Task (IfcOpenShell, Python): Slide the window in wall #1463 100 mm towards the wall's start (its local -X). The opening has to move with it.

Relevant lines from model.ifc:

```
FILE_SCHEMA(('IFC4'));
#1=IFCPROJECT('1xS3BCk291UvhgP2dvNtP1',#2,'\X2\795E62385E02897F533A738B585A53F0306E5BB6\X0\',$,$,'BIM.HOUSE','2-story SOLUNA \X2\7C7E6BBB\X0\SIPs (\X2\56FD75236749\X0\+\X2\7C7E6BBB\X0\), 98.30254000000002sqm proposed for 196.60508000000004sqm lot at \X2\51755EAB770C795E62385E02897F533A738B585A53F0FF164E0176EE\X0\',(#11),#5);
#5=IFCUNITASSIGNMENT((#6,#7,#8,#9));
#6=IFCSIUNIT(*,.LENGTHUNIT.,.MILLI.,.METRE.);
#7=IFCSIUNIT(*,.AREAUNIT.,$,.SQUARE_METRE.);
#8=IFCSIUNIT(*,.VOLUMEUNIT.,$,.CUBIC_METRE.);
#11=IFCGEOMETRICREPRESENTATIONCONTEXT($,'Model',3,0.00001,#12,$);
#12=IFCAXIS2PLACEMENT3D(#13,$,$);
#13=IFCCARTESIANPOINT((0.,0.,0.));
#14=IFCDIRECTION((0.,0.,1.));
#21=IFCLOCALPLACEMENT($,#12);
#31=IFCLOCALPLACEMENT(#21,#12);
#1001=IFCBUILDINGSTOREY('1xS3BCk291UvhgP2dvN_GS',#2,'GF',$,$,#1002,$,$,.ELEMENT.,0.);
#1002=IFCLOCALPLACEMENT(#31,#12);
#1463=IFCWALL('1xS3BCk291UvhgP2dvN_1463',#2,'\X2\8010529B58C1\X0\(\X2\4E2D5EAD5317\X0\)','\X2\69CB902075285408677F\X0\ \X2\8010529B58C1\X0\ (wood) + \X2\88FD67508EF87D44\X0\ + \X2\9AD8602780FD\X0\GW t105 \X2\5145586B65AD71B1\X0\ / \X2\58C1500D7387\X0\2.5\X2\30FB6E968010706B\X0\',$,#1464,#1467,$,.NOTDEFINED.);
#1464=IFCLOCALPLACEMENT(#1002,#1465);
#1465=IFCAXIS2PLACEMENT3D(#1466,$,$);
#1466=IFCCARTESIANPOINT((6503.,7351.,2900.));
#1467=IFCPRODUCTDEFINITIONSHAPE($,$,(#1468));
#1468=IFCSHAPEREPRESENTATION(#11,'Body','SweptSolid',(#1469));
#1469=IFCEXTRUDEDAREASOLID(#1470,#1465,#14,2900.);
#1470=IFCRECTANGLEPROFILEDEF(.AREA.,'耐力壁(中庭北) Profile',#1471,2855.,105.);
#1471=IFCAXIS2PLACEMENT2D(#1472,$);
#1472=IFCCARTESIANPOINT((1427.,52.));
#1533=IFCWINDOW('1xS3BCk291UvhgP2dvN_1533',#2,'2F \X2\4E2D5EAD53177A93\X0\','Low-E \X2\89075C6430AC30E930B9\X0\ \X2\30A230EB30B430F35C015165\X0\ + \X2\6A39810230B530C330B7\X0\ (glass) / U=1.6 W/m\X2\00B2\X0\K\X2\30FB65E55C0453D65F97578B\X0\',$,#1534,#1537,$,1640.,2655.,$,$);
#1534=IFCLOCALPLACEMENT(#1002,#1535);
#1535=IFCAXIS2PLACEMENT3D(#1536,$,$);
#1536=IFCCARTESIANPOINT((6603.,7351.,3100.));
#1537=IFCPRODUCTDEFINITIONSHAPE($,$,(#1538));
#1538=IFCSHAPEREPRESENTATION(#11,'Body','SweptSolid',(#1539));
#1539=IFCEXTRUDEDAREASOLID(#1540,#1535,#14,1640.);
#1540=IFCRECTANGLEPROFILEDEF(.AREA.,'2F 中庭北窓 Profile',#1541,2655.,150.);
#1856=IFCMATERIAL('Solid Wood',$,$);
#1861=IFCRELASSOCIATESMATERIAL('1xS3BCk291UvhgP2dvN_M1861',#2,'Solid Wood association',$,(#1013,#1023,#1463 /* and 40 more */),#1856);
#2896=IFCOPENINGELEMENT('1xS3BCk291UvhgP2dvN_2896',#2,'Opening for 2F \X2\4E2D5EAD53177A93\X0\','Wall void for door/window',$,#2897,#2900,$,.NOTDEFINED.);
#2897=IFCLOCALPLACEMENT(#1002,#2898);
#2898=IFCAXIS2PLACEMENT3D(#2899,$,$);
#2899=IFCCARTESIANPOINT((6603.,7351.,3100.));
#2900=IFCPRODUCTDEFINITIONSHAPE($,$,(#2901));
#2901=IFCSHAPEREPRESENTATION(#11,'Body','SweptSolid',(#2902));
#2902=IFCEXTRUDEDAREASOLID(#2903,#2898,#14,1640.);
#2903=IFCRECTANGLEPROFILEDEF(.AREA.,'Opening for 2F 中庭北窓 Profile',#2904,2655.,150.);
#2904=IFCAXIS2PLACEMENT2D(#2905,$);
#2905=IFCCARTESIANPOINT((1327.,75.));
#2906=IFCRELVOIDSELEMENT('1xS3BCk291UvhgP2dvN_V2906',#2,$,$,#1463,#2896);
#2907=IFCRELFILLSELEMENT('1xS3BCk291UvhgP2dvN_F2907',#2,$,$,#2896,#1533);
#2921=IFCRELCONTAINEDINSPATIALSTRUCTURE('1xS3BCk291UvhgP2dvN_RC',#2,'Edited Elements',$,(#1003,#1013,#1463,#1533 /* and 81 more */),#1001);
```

```python
import ifcopenshell
import ifcopenshell.api.geometry
import ifcopenshell.util.placement

model = ifcopenshell.open("model.ifc")

window = model.by_id(1533)
opening = window.FillsVoids[0].RelatingOpeningElement
wall = opening.VoidsElements[0].RelatingBuildingElement

wall_matrix = ifcopenshell.util.placement.get_local_placement(wall.ObjectPlacement)
shift = wall_matrix[:3, 0] * -100.0
before = ifcopenshell.util.placement.get_local_placement(window.ObjectPlacement)[:3, 3].copy()

# The window is not placed relative to its opening, so move both.
for product in (opening, window):
    matrix = ifcopenshell.util.placement.get_local_placement(product.ObjectPlacement)
    matrix[:3, 3] += shift
    ifcopenshell.api.geometry.edit_object_placement(model, product=product, matrix=matrix, is_si=False)

after = ifcopenshell.util.placement.get_local_placement(window.ObjectPlacement)[:3, 3]
print("window moved by", (after - before).round(3) + 0.0)

model.write("model-out.ifc")
```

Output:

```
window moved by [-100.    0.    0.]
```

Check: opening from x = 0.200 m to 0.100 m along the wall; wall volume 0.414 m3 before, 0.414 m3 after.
